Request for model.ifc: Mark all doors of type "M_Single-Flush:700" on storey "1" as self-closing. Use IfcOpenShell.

First a look at what the model holds.

```python
import ifcopenshell
import ifcopenshell.util.element

model = ifcopenshell.open("model.ifc")
print(model.schema)
storey = next(s for s in model.by_type("IfcBuildingStorey") if s.Name == "1")
doors = [e for e in ifcopenshell.util.element.get_decomposition(storey) if e.is_a("IfcDoor")]
seen = {}
for e in doors:
    element_type = ifcopenshell.util.element.get_type(e)
    key = (element_type.Name if element_type != e and element_type else None, ifcopenshell.util.element.get_pset(e, "Pset_DoorCommon", "SelfClosing"))
    seen[key] = seen.get(key, 0) + 1
for (name, value), count in sorted(seen.items(), key=str):
    print(count, "x", name, "|", value)
```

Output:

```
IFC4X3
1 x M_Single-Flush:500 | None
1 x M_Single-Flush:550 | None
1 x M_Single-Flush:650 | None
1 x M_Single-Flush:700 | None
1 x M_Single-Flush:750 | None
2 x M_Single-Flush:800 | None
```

```python
import ifcopenshell
import ifcopenshell.api.pset
import ifcopenshell.util.element

model = ifcopenshell.open("model.ifc")

storey = next(s for s in model.by_type("IfcBuildingStorey") if s.Name == "1")
doors = [e for e in ifcopenshell.util.element.get_decomposition(storey) if e.is_a("IfcDoor")]

count = 0
for e in doors:
    element_type = ifcopenshell.util.element.get_type(e)
    if element_type in (None, e) or element_type.Name != "M_Single-Flush:700":
        continue
    # add_pset returns the element's existing set when there is one.
    pset = ifcopenshell.api.pset.add_pset(model, product=e, name="Pset_DoorCommon")
    ifcopenshell.api.pset.edit_pset(model, pset=pset, properties={"SelfClosing": True})
    count += 1

print(count, "doors updated")

model.write("model_edited.ifc")
```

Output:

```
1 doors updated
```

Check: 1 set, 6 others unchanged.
